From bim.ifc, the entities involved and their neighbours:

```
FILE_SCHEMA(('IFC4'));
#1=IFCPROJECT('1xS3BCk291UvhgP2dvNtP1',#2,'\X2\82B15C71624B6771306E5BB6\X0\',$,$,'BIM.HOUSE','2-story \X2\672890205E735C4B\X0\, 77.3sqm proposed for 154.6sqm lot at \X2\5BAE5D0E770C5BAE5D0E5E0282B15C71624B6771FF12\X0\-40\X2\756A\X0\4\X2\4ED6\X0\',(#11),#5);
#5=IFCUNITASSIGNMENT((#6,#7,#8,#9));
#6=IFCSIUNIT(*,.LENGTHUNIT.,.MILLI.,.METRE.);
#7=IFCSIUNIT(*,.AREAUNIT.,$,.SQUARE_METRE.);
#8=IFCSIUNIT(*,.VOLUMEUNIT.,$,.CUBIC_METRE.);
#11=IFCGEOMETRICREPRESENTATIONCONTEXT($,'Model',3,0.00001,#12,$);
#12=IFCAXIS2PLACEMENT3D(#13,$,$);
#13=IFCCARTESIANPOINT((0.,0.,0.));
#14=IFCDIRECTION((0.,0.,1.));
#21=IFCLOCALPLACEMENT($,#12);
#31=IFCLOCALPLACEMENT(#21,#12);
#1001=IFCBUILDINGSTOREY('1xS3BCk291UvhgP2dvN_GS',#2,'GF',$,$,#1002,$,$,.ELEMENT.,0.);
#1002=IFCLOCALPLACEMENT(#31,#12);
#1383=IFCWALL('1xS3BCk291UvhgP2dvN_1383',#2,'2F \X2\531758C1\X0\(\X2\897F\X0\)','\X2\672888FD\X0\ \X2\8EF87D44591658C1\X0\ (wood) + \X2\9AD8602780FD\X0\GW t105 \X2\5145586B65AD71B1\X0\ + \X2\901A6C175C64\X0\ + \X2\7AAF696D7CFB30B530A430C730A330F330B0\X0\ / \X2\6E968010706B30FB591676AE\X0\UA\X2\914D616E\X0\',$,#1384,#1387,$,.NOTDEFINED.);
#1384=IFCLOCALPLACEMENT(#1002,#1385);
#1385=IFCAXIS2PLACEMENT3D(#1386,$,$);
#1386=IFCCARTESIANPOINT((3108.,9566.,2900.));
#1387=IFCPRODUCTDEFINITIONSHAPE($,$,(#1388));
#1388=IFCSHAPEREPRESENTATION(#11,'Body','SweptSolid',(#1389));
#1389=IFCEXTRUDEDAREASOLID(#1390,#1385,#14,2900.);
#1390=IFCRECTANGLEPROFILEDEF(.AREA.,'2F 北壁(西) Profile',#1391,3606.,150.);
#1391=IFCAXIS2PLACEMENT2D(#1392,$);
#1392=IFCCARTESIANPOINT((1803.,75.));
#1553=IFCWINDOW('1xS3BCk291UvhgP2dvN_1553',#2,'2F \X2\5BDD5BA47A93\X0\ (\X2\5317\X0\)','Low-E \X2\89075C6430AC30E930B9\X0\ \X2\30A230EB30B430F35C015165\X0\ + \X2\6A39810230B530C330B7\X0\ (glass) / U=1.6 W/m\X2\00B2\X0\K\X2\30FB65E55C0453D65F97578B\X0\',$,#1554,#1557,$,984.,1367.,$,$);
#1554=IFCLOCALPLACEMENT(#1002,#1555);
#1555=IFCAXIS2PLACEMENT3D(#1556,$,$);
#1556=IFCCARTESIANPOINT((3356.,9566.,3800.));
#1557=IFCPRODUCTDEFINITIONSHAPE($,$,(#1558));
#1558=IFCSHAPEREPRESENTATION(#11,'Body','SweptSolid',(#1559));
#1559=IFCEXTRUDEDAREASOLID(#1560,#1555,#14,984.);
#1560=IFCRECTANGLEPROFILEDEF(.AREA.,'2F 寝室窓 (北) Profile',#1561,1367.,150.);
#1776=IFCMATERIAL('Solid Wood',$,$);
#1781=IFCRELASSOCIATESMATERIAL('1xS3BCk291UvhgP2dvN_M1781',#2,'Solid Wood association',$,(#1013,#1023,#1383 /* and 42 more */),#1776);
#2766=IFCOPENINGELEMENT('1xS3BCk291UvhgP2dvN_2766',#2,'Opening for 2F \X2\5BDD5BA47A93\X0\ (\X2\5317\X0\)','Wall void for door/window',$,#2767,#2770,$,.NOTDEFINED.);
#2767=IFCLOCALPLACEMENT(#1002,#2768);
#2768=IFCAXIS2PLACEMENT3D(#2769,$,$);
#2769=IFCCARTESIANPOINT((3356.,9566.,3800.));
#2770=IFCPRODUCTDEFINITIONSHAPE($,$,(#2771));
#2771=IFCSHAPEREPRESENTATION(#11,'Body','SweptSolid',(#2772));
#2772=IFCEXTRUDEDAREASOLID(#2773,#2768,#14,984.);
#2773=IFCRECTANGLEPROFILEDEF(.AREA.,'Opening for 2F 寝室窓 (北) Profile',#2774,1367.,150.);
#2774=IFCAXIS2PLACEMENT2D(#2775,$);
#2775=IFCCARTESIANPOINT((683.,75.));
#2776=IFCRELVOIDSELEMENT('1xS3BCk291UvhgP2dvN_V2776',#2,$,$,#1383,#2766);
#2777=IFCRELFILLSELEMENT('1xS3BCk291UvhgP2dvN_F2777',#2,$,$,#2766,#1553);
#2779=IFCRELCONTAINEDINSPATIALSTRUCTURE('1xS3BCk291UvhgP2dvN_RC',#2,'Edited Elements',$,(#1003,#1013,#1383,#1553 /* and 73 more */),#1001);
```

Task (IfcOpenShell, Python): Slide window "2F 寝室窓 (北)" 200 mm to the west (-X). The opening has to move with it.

```python
import ifcopenshell
import ifcopenshell.api.geometry
import ifcopenshell.util.placement
import ifcopenshell.util.unit

model = ifcopenshell.open("bim.ifc")
unit_scale = ifcopenshell.util.unit.calculate_unit_scale(model)

window = model.by_guid("1xS3BCk291UvhgP2dvN_1553")
opening = window.FillsVoids[0].RelatingOpeningElement
wall = opening.VoidsElements[0].RelatingBuildingElement

wall_matrix = ifcopenshell.util.placement.get_local_placement(wall.ObjectPlacement)
shift = wall_matrix[:3, 0] * -0.2 / unit_scale
before = ifcopenshell.util.placement.get_local_placement(window.ObjectPlacement)[:3, 3].copy()

# The window is not placed relative to its opening, so move both.
for product in (opening, window):
    matrix = ifcopenshell.util.placement.get_local_placement(product.ObjectPlacement)
    matrix[:3, 3] += shift
    ifcopenshell.api.geometry.edit_object_placement(model, product=product, matrix=matrix, is_si=False)

after = ifcopenshell.util.placement.get_local_placement(window.ObjectPlacement)[:3, 3]
print("window moved by", (after - before).round(3) + 0.0)

model.write("bim_v2.ifc")
```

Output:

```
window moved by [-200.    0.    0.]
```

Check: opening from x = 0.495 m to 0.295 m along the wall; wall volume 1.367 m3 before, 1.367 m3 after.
